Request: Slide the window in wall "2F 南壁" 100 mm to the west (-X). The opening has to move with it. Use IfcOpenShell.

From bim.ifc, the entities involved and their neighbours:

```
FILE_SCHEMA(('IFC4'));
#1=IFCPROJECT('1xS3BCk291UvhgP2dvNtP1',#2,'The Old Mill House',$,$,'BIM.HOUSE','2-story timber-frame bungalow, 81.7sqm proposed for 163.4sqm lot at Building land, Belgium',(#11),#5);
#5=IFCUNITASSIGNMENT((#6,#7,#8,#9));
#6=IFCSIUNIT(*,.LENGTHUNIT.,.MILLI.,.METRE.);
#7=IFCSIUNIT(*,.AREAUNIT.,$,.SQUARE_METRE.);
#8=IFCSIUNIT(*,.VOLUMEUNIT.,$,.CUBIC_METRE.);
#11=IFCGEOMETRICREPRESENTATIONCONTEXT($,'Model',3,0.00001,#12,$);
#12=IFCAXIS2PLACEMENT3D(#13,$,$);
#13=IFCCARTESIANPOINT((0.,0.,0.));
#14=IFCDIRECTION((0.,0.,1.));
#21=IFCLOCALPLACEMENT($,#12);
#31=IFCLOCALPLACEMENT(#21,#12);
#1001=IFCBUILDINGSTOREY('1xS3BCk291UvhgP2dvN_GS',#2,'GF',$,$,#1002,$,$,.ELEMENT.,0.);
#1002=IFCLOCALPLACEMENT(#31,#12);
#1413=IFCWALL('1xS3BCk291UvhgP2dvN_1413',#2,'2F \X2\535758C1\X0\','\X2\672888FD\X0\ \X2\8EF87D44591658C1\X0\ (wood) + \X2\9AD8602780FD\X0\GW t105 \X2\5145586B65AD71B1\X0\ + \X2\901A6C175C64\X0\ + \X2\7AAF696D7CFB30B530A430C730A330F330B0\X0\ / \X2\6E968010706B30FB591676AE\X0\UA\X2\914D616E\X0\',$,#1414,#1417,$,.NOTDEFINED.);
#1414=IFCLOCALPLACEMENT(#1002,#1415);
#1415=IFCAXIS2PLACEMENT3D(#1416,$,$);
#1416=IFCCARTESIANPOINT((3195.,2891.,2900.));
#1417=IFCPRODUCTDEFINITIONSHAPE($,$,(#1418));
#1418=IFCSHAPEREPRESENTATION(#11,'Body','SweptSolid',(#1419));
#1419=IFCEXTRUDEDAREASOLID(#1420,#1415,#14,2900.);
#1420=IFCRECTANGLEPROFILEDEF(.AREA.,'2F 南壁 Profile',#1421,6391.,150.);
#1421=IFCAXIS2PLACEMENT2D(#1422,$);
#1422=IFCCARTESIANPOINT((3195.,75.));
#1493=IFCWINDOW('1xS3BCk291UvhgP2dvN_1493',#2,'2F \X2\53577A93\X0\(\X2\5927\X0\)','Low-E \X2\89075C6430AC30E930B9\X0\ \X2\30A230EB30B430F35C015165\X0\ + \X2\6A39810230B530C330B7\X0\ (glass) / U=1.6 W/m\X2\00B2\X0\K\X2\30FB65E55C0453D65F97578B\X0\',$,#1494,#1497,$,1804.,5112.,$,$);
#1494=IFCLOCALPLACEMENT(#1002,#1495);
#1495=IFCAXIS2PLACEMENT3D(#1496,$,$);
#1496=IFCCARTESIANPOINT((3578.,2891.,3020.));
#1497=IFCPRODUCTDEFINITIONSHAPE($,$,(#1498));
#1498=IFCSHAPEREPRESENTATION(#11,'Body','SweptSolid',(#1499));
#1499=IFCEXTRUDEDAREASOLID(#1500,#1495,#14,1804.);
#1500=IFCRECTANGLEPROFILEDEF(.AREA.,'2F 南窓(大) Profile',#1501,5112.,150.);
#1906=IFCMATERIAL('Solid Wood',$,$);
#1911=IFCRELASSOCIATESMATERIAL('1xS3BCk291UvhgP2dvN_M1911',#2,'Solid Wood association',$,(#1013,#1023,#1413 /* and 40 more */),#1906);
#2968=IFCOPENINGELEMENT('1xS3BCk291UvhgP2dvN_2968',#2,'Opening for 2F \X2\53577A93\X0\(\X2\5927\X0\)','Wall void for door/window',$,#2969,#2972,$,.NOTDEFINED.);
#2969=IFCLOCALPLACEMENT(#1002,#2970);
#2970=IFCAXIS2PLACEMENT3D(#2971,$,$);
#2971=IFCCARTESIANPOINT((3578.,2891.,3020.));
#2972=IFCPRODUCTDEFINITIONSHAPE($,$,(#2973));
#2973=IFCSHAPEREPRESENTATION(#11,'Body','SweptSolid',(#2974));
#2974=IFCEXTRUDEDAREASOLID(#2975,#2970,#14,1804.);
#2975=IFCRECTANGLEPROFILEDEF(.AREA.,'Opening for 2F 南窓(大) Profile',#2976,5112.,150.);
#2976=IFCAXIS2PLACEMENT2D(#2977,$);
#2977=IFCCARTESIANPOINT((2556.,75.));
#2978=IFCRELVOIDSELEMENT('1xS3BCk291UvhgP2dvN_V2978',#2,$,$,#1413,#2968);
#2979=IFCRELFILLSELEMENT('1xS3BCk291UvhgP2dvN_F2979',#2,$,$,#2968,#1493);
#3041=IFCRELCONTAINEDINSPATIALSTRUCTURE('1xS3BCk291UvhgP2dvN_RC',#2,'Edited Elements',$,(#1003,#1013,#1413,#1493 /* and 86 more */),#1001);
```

```python
import ifcopenshell
import ifcopenshell.api.geometry
import ifcopenshell.util.placement
import ifcopenshell.util.unit

model = ifcopenshell.open("bim.ifc")
unit_scale = ifcopenshell.util.unit.calculate_unit_scale(model)

window = model.by_guid("1xS3BCk291UvhgP2dvN_1493")
opening = window.FillsVoids[0].RelatingOpeningElement
wall = opening.VoidsElements[0].RelatingBuildingElement

wall_matrix = ifcopenshell.util.placement.get_local_placement(wall.ObjectPlacement)
shift = wall_matrix[:3, 0] * -0.1 / unit_scale
before = ifcopenshell.util.placement.get_local_placement(window.ObjectPlacement)[:3, 3].copy()

# The window is not placed relative to its opening, so move both.
for product in (opening, window):
    matrix = ifcopenshell.util.placement.get_local_placement(product.ObjectPlacement)
    matrix[:3, 3] += shift
    ifcopenshell.api.geometry.edit_object_placement(model, product=product, matrix=matrix, is_si=False)

after = ifcopenshell.util.placement.get_local_placement(window.ObjectPlacement)[:3, 3]
print("window moved by", (after - before).round(3) + 0.0)

model.write("bim_v2.ifc")
```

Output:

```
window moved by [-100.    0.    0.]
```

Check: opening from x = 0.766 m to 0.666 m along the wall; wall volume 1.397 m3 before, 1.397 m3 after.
